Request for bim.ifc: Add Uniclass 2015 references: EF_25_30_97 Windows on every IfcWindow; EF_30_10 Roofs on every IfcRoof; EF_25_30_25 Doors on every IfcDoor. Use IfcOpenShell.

First a look at what the model holds.

```python
import ifcopenshell

model = ifcopenshell.open("bim.ifc")
print(model.schema)
print("classifications:", [c.Name for c in model.by_type("IfcClassification")])
for ifc_class in ("IfcDoor", "IfcRoof", "IfcStair", "IfcWall", "IfcWindow"):
    print(ifc_class, len(model.by_type(ifc_class)))
```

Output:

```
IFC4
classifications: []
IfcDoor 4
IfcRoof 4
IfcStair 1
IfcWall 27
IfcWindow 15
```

```python
import ifcopenshell
import ifcopenshell.api.classification

model = ifcopenshell.open("bim.ifc")

system = ifcopenshell.api.classification.add_classification(model, classification="Uniclass 2015")

codes = {
    "IfcWindow": ("EF_25_30_97", "Windows"),
    "IfcRoof": ("EF_30_10", "Roofs"),
    "IfcDoor": ("EF_25_30_25", "Doors"),
}
for ifc_class, (code, name) in codes.items():
    products = model.by_type(ifc_class)
    ifcopenshell.api.classification.add_reference(
        model, products=products, classification=system, identification=code, name=name
    )
    print(code, len(products))

model.write("bim_updated.ifc")
```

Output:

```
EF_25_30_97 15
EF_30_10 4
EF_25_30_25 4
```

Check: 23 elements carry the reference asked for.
